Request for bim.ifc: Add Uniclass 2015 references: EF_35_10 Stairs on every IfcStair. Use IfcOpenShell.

First a look at what the model holds.

```python
import ifcopenshell

model = ifcopenshell.open("bim.ifc")
print(model.schema)
print("classifications:", [c.Name for c in model.by_type("IfcClassification")])
for ifc_class in ("IfcDoor", "IfcRoof", "IfcStair", "IfcWall", "IfcWindow"):
    print(ifc_class, len(model.by_type(ifc_class)))
```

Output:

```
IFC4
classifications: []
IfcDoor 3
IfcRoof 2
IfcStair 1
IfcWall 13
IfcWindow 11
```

```python
import ifcopenshell
import ifcopenshell.api.classification

model = ifcopenshell.open("bim.ifc")

system = ifcopenshell.api.classification.add_classification(model, classification="Uniclass 2015")

codes = {
    "IfcStair": ("EF_35_10", "Stairs"),
}
for ifc_class, (code, name) in codes.items():
    products = model.by_type(ifc_class)
    ifcopenshell.api.classification.add_reference(
        model, products=products, classification=system, identification=code, name=name
    )
    print(code, len(products))

model.write("bim_updated.ifc")
```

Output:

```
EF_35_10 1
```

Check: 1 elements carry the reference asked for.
